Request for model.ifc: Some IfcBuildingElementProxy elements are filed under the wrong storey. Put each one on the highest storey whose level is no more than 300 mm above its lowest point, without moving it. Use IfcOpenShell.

First a look at what the model holds.

```python
import ifcopenshell
import ifcopenshell.util.element
import ifcopenshell.util.placement

model = ifcopenshell.open("model.ifc")
print(model.schema)
for storey in model.by_type("IfcBuildingStorey"):
    level = ifcopenshell.util.placement.get_storey_elevation(storey)
    count = sum(e.is_a("IfcBuildingElementProxy") for e in ifcopenshell.util.element.get_contained(storey))
    print(storey.id(), storey.Name, round(level, 3), count, sep=" | ")
```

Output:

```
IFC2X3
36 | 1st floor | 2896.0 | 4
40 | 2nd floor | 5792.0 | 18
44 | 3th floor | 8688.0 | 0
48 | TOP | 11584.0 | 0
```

```python
import ifcopenshell
import ifcopenshell.api.spatial
import ifcopenshell.geom
import ifcopenshell.util.element
import ifcopenshell.util.placement
import ifcopenshell.util.shape
import ifcopenshell.util.unit

model = ifcopenshell.open("model.ifc")
unit_scale = ifcopenshell.util.unit.calculate_unit_scale(model)
settings = ifcopenshell.geom.settings()

levels = sorted(
    ((ifcopenshell.util.placement.get_storey_elevation(s) * unit_scale, s) for s in model.by_type("IfcBuildingStorey")),
    key=lambda pair: pair[0],
)

for e in model.by_type("IfcBuildingElementProxy"):
    current = e.ContainedInStructure[0].RelatingStructure if e.ContainedInStructure else None
    if current is None or not current.is_a("IfcBuildingStorey"):
        continue
    shape = ifcopenshell.geom.create_shape(settings, e)
    bottom = ifcopenshell.util.shape.get_shape_bottom_elevation(shape, shape.geometry)
    below = [s for level, s in levels if level <= bottom + 0.3]
    storey = below[-1] if below else levels[0][1]
    if storey != current:
        # assign_container keeps the world position.
        ifcopenshell.api.spatial.assign_container(model, products=[e], relating_structure=storey)
        print(e.id(), current.Name, "->", storey.Name)

model.write("model_edited.ifc")
```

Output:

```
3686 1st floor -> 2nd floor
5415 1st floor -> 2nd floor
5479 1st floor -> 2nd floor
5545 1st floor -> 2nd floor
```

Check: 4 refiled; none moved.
